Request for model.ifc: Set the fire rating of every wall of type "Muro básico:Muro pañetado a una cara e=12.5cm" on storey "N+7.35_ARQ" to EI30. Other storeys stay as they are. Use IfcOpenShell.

First a look at what the model holds.

```python
import ifcopenshell
import ifcopenshell.util.element

model = ifcopenshell.open("model.ifc")
print(model.schema)
storey = next(s for s in model.by_type("IfcBuildingStorey") if s.Name == "N+7.35_ARQ")
walls = [e for e in ifcopenshell.util.element.get_decomposition(storey) if e.is_a("IfcWall")]
seen = {}
for e in walls:
    element_type = ifcopenshell.util.element.get_type(e)
    key = (element_type.Name if element_type != e and element_type else None, ifcopenshell.util.element.get_pset(e, "Pset_WallCommon", "FireRating"))
    seen[key] = seen.get(key, 0) + 1
for (name, value), count in sorted(seen.items(), key=str):
    print(count, "x", name, "|", value)
```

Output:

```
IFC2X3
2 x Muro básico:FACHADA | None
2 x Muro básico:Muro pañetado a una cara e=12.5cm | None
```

```python
import ifcopenshell
import ifcopenshell.api.pset
import ifcopenshell.util.element

model = ifcopenshell.open("model.ifc")

storey = next(s for s in model.by_type("IfcBuildingStorey") if s.Name == "N+7.35_ARQ")
walls = [e for e in ifcopenshell.util.element.get_decomposition(storey) if e.is_a("IfcWall")]

count = 0
for e in walls:
    element_type = ifcopenshell.util.element.get_type(e)
    if element_type in (None, e) or element_type.Name != "Muro básico:Muro pañetado a una cara e=12.5cm":
        continue
    # add_pset returns the element's existing set when there is one.
    pset = ifcopenshell.api.pset.add_pset(model, product=e, name="Pset_WallCommon")
    ifcopenshell.api.pset.edit_pset(model, pset=pset, properties={"FireRating": "EI30"})
    count += 1

print(count, "walls updated")

model.write("model_rev.ifc")
```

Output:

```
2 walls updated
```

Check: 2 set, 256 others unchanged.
